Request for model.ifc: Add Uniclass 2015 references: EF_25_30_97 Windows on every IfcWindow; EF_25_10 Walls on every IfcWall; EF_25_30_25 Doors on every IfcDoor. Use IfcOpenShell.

First a look at what the model holds.

```python
import ifcopenshell

model = ifcopenshell.open("model.ifc")
print(model.schema)
print("classifications:", [c.Name for c in model.by_type("IfcClassification")])
for ifc_class in ("IfcDoor", "IfcRoof", "IfcStair", "IfcWall", "IfcWindow"):
    print(ifc_class, len(model.by_type(ifc_class)))
```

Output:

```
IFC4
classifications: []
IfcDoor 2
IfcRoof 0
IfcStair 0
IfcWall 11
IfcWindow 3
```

```python
import ifcopenshell
import ifcopenshell.api.classification

model = ifcopenshell.open("model.ifc")

system = ifcopenshell.api.classification.add_classification(model, classification="Uniclass 2015")

codes = {
    "IfcWindow": ("EF_25_30_97", "Windows"),
    "IfcWall": ("EF_25_10", "Walls"),
    "IfcDoor": ("EF_25_30_25", "Doors"),
}
for ifc_class, (code, name) in codes.items():
    products = model.by_type(ifc_class)
    ifcopenshell.api.classification.add_reference(
        model, products=products, classification=system, identification=code, name=name
    )
    print(code, len(products))

model.write("model_v2.ifc")
```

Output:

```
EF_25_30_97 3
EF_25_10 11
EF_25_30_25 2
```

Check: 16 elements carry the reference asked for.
